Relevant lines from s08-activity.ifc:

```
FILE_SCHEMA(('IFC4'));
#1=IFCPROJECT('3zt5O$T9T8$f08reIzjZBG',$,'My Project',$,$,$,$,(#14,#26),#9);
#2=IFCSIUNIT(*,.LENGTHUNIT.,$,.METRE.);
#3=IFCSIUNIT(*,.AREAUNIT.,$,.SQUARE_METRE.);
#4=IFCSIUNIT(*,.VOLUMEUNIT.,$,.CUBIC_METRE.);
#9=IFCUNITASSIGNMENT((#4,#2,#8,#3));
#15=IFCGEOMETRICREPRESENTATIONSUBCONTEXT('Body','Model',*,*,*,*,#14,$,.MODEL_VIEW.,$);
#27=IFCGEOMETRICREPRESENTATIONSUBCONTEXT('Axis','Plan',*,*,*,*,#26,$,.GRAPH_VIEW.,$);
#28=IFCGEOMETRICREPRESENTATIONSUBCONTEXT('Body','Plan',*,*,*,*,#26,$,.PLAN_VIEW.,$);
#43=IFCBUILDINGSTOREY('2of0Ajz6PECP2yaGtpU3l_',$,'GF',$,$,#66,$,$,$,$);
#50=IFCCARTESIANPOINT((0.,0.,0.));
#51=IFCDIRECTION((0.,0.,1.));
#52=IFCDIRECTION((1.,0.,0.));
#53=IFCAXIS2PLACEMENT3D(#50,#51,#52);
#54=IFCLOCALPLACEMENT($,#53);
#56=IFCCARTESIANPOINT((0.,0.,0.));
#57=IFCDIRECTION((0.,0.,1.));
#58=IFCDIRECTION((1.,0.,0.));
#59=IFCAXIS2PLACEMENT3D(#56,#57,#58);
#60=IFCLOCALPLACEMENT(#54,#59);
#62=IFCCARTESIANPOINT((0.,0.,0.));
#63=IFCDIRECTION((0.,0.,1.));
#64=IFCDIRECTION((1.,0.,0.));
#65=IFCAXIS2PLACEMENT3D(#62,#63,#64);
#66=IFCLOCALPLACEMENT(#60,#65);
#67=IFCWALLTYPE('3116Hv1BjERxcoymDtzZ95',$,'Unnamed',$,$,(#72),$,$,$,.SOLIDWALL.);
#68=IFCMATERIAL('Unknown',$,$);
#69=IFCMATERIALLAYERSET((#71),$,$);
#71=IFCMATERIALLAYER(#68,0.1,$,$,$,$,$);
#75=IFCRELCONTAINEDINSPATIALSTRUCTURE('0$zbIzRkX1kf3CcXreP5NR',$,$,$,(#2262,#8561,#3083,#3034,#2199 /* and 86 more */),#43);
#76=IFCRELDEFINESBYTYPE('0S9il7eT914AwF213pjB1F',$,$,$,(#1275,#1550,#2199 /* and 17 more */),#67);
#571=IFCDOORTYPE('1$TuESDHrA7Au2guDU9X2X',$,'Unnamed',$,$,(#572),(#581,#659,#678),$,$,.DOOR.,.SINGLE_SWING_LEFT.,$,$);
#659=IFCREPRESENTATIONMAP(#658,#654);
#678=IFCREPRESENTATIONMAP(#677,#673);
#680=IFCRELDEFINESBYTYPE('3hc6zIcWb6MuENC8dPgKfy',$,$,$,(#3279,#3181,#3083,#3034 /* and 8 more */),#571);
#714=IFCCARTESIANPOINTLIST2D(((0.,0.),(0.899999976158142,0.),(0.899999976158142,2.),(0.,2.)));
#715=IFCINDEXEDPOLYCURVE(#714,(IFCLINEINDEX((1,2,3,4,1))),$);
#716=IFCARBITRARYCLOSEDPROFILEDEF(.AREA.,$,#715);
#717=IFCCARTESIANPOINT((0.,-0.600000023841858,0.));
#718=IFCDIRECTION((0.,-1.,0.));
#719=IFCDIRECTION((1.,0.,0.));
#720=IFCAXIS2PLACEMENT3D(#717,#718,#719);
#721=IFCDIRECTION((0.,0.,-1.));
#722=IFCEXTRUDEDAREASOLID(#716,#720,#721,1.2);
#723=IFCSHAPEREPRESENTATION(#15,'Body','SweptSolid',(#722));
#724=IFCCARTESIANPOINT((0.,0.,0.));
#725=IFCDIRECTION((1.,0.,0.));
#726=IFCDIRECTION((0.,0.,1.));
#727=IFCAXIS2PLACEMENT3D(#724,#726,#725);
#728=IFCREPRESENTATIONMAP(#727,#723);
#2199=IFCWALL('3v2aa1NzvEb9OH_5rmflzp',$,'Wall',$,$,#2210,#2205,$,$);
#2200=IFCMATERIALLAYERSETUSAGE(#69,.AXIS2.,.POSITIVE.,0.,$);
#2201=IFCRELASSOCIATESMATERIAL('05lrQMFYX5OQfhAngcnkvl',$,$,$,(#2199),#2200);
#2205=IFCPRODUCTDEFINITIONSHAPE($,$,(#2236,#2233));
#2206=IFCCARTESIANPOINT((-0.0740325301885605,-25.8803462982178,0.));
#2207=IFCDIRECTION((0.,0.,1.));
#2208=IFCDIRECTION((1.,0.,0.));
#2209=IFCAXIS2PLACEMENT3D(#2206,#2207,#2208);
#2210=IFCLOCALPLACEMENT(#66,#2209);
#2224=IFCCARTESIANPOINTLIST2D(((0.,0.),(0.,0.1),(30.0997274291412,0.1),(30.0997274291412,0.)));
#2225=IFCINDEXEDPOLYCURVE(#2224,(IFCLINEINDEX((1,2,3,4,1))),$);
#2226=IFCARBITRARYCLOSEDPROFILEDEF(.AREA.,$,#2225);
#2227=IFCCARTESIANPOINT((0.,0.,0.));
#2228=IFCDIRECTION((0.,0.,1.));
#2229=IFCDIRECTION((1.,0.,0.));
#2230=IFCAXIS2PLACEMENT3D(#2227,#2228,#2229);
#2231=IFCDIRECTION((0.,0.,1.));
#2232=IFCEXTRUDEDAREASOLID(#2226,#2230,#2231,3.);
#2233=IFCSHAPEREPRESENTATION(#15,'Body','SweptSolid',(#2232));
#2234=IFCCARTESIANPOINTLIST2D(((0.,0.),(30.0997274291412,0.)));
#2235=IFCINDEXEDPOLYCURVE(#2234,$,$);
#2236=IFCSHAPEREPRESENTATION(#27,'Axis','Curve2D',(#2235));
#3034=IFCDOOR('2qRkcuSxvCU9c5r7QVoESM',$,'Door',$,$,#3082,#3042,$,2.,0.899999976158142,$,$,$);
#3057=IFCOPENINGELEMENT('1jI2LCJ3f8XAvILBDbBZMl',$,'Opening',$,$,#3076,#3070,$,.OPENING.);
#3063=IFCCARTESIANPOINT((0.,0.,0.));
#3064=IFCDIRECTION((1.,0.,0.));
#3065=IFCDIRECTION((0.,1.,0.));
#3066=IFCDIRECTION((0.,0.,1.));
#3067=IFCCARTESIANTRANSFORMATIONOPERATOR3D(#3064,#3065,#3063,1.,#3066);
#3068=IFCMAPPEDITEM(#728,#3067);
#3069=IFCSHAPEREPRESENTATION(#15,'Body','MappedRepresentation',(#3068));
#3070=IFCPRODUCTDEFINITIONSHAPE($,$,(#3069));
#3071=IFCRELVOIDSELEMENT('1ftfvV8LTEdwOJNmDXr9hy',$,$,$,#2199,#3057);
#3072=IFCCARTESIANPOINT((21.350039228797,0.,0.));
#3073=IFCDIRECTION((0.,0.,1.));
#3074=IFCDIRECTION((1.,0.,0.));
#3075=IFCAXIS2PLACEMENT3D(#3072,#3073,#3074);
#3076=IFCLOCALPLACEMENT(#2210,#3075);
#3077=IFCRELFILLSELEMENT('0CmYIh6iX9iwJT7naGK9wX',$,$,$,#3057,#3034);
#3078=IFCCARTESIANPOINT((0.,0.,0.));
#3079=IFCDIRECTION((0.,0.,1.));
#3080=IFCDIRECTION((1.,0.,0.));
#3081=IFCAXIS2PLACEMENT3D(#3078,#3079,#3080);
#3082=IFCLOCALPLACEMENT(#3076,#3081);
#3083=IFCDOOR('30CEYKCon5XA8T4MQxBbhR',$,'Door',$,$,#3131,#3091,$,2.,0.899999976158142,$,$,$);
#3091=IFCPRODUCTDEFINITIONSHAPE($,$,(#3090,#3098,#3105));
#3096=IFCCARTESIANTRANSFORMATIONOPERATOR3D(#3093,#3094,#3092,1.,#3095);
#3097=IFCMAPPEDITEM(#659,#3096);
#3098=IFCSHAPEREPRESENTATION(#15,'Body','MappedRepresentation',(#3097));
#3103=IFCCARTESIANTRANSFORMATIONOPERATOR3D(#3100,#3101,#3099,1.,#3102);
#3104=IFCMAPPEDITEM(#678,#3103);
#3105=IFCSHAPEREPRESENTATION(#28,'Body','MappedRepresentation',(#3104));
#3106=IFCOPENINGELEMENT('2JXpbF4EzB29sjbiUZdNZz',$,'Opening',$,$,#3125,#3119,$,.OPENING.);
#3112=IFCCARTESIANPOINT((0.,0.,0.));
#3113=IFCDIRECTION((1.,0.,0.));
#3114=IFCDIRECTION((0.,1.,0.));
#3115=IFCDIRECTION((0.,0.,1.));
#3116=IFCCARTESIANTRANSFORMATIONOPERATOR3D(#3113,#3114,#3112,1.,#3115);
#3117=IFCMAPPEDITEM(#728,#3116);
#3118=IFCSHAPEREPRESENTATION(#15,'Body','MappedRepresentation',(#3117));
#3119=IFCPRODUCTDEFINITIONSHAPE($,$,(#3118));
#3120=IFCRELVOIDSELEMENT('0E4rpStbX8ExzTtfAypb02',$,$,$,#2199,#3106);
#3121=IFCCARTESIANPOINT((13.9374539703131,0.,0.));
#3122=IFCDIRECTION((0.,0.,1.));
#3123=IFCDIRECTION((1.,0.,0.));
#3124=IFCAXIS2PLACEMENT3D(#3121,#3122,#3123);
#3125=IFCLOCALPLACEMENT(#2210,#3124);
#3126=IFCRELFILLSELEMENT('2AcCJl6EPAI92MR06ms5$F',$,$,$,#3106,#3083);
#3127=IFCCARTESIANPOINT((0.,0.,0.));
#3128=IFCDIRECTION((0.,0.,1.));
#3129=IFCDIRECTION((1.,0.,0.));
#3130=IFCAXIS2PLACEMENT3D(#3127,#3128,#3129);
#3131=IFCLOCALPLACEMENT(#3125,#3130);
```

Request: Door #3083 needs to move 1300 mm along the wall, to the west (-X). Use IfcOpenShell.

```python
import ifcopenshell
import ifcopenshell.api.geometry
import ifcopenshell.util.placement

model = ifcopenshell.open("s08-activity.ifc")

door = model.by_guid("30CEYKCon5XA8T4MQxBbhR")
opening = door.FillsVoids[0].RelatingOpeningElement
wall = opening.VoidsElements[0].RelatingBuildingElement

wall_matrix = ifcopenshell.util.placement.get_local_placement(wall.ObjectPlacement)
shift = wall_matrix[:3, 0] * -1.3
before = ifcopenshell.util.placement.get_local_placement(door.ObjectPlacement)[:3, 3].copy()

# The door is placed relative to its opening, so it follows when the opening moves.
matrix = ifcopenshell.util.placement.get_local_placement(opening.ObjectPlacement)
matrix[:3, 3] += shift
ifcopenshell.api.geometry.edit_object_placement(
    model, product=opening, matrix=matrix, is_si=False, should_transform_children=True
)

after = ifcopenshell.util.placement.get_local_placement(door.ObjectPlacement)[:3, 3]
print("door moved by", (after - before).round(3) + 0.0)

model.write("s08-activity_updated.ifc")
```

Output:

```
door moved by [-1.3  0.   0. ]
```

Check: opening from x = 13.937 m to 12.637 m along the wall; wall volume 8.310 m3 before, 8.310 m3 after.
